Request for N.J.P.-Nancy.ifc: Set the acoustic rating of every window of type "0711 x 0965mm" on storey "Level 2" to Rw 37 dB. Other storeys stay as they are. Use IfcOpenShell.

First a look at what the model holds.

```python
import ifcopenshell
import ifcopenshell.util.element

model = ifcopenshell.open("N.J.P.-Nancy.ifc")
print(model.schema)
storey = next(s for s in model.by_type("IfcBuildingStorey") if s.Name == "Level 2")
windows = [e for e in ifcopenshell.util.element.get_decomposition(storey) if e.is_a("IfcWindow")]
seen = {}
for e in windows:
    element_type = ifcopenshell.util.element.get_type(e)
    key = (element_type.Name if element_type != e and element_type else None, ifcopenshell.util.element.get_pset(e, "Pset_WindowCommon", "AcousticRating"))
    seen[key] = seen.get(key, 0) + 1
for (name, value), count in sorted(seen.items(), key=str):
    print(count, "x", name, "|", value)
```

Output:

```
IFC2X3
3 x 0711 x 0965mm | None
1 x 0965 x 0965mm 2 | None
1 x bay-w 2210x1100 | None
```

```python
import ifcopenshell
import ifcopenshell.api.pset
import ifcopenshell.util.element

model = ifcopenshell.open("N.J.P.-Nancy.ifc")

storey = next(s for s in model.by_type("IfcBuildingStorey") if s.Name == "Level 2")
windows = [e for e in ifcopenshell.util.element.get_decomposition(storey) if e.is_a("IfcWindow")]

count = 0
for e in windows:
    element_type = ifcopenshell.util.element.get_type(e)
    if element_type in (None, e) or element_type.Name != "0711 x 0965mm":
        continue
    # add_pset returns the element's existing set when there is one.
    pset = ifcopenshell.api.pset.add_pset(model, product=e, name="Pset_WindowCommon")
    ifcopenshell.api.pset.edit_pset(model, pset=pset, properties={"AcousticRating": "Rw 37 dB"})
    count += 1

print(count, "windows updated")

model.write("N.J.P.-Nancy_rev.ifc")
```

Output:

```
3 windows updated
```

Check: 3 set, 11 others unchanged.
